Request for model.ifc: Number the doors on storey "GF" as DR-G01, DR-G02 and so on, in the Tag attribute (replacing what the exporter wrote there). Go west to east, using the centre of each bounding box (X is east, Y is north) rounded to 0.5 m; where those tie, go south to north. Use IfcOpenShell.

First a look at what the model holds.

```python
import ifcopenshell
import ifcopenshell.util.element
import ifcopenshell.util.placement

model = ifcopenshell.open("model.ifc")
print(model.schema)
storey = next(s for s in model.by_type("IfcBuildingStorey") if s.Name == "GF")
doors = [e for e in ifcopenshell.util.element.get_decomposition(storey) if e.is_a("IfcDoor")]
for e in sorted(doors, key=lambda e: e.id()):
    origin = ifcopenshell.util.placement.get_local_placement(e.ObjectPlacement)[:3, 3]
    print(e.id(), e.Tag, e.Name, origin.round(2) + 0.0, sep=" | ")
```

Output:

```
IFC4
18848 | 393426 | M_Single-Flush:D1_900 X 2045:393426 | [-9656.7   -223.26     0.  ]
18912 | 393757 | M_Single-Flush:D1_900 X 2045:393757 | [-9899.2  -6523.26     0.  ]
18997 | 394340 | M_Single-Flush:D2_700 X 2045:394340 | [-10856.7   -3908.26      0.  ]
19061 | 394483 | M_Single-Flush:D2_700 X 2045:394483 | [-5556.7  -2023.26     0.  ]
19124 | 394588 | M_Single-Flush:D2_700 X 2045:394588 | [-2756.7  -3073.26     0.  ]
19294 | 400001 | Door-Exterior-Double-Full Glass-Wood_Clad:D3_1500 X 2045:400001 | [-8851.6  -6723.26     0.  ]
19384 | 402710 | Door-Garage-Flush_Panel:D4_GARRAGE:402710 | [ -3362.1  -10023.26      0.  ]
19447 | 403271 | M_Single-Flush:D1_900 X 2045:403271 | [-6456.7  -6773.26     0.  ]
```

```python
import ifcopenshell
import ifcopenshell.geom
import ifcopenshell.util.element
import ifcopenshell.util.shape

model = ifcopenshell.open("model.ifc")
settings = ifcopenshell.geom.settings()
settings.set("use-world-coords", True)


def centre(element):
    shape = ifcopenshell.geom.create_shape(settings, element)
    return ifcopenshell.util.shape.get_bbox_centroid(shape.geometry)


storey = next(s for s in model.by_type("IfcBuildingStorey") if s.Name == "GF")
doors = [e for e in ifcopenshell.util.element.get_decomposition(storey) if e.is_a("IfcDoor")]

# Insertion points can sit at a corner or the storey origin, so sort by the geometry (in metres).
centres = {e: centre(e) for e in doors}
doors.sort(key=lambda e: (round(centres[e][0] / 0.5), centres[e][1]))

for i, e in enumerate(doors, start=1):
    number = f"DR-G{i:02d}"
    e.Tag = number
    print(e.id(), number)

model.write("model-out.ifc")
```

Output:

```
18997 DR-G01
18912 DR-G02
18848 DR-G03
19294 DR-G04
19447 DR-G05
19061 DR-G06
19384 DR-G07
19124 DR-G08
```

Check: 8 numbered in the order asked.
